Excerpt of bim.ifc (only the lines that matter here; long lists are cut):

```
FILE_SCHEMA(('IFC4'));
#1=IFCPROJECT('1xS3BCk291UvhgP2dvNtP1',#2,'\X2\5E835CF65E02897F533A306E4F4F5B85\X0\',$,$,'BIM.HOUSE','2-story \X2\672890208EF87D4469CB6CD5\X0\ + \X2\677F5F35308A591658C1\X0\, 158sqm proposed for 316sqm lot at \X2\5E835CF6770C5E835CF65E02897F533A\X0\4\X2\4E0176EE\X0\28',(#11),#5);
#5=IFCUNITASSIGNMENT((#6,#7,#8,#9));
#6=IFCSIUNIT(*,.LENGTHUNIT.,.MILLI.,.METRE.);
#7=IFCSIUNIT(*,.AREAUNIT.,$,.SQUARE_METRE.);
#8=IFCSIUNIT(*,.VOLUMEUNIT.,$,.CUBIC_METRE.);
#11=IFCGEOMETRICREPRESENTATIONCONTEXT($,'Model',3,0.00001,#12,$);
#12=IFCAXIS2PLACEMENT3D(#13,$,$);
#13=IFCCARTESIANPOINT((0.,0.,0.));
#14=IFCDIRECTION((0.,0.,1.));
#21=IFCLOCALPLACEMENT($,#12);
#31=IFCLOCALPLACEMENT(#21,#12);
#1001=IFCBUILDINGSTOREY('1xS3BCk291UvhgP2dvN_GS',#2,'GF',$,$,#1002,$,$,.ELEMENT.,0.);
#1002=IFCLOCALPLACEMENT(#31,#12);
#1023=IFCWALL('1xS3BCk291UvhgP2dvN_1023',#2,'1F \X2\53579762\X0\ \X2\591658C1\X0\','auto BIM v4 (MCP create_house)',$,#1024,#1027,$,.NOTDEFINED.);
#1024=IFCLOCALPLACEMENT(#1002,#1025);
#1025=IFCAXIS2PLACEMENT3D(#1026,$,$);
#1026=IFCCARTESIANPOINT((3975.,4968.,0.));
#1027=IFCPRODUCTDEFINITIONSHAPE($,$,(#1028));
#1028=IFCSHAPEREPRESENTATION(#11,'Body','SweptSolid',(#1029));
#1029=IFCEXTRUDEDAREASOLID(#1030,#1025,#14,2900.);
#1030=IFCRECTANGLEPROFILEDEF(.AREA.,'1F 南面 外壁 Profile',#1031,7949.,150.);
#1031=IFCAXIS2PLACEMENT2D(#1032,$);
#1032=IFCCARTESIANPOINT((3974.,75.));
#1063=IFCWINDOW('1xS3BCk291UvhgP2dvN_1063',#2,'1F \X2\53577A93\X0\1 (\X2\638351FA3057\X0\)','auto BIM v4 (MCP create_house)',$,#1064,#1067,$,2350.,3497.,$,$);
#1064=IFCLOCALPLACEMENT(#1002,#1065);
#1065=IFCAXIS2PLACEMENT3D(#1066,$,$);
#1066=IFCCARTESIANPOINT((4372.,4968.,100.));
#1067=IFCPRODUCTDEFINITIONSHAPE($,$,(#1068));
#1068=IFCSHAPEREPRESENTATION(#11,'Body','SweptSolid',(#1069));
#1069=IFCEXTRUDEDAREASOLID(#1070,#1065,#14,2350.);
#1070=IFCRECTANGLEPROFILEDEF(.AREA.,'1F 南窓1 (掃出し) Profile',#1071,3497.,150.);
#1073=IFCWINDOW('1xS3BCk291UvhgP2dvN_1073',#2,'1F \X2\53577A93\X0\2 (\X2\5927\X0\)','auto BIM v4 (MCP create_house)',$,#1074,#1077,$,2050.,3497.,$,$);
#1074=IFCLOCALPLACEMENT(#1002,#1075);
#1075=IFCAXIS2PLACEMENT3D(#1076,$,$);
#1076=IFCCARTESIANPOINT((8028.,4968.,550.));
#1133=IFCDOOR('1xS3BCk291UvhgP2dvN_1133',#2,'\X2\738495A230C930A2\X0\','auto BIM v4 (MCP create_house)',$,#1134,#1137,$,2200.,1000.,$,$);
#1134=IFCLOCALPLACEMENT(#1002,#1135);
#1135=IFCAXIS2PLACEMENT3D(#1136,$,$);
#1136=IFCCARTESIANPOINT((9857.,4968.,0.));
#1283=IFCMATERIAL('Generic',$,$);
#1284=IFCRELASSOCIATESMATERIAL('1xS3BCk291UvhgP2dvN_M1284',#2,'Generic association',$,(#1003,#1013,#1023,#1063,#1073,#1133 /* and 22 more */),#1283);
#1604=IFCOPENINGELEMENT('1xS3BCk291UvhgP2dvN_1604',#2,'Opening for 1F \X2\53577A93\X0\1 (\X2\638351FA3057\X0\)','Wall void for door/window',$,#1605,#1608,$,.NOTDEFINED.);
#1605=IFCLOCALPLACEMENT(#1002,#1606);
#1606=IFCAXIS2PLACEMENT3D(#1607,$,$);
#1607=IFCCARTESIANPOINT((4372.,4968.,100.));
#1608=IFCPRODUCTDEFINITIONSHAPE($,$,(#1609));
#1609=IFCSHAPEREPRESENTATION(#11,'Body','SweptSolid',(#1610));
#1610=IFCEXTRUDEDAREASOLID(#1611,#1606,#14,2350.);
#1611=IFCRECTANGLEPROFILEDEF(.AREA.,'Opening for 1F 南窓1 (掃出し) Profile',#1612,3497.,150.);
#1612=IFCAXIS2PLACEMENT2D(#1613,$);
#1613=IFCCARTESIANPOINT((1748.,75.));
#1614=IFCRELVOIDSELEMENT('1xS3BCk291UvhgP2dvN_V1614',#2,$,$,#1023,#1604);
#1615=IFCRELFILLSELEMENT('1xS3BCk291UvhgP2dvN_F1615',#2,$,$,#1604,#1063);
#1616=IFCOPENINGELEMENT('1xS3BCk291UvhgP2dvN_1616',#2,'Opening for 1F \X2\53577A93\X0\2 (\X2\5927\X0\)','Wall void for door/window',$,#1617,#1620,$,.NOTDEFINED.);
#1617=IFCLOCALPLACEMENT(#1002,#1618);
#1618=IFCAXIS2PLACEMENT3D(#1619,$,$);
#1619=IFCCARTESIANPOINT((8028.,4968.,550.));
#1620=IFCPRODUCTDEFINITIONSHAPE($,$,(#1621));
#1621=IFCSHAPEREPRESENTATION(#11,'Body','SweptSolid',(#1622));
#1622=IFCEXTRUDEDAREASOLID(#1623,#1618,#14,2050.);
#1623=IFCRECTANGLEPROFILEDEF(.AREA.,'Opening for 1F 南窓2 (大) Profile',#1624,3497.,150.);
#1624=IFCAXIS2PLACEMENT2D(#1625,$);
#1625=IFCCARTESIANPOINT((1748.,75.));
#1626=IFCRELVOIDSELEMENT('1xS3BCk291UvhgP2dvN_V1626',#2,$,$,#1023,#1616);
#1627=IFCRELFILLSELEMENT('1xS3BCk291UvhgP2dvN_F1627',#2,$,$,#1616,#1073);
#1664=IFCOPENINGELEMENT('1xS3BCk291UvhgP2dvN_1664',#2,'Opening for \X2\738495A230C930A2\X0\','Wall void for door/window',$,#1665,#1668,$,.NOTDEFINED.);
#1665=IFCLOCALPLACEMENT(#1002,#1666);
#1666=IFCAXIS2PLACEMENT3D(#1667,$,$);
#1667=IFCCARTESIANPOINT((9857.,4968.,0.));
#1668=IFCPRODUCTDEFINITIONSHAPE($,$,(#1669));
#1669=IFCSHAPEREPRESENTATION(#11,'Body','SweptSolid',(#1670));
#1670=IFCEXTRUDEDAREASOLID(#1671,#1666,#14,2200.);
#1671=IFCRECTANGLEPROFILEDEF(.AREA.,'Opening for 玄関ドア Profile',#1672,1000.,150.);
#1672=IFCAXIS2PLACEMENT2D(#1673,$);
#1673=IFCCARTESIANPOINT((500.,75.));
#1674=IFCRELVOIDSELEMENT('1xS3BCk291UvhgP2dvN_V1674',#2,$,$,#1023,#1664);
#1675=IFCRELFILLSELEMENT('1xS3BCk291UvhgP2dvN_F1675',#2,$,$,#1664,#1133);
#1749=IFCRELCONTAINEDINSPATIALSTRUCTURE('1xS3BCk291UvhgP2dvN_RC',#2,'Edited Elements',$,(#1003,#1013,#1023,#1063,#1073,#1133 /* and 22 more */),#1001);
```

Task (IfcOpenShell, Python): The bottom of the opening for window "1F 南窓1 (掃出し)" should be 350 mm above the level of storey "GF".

```python
import numpy as np
import ifcopenshell
import ifcopenshell.api.geometry
import ifcopenshell.geom
import ifcopenshell.util.element
import ifcopenshell.util.placement
import ifcopenshell.util.shape
import ifcopenshell.util.unit

model = ifcopenshell.open("bim.ifc")
unit_scale = ifcopenshell.util.unit.calculate_unit_scale(model)

window = model.by_id(1063)
opening = window.FillsVoids[0].RelatingOpeningElement
storey = ifcopenshell.util.element.get_container(window, ifc_class="IfcBuildingStorey")
level = ifcopenshell.util.placement.get_local_placement(storey.ObjectPlacement)[2, 3]

# The opening's origin need not be at the sill, so measure its lowest point.
shape = ifcopenshell.geom.create_shape(ifcopenshell.geom.settings(), opening)
bottom = ifcopenshell.util.shape.get_shape_bottom_elevation(shape, shape.geometry) / unit_scale
dz = level + 0.35 / unit_scale - bottom

shift = np.array([0.0, 0.0, dz])
# The window is not placed relative to its opening, so move both.
for product in (opening, window):
    matrix = ifcopenshell.util.placement.get_local_placement(product.ObjectPlacement)
    matrix[:3, 3] += shift
    ifcopenshell.api.geometry.edit_object_placement(model, product=product, matrix=matrix, is_si=False)

print(f"moved by {dz * unit_scale:+.3f} m")

model.write("bim_edited.ifc")
```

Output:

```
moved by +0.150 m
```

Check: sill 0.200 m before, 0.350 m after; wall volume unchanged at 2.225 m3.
